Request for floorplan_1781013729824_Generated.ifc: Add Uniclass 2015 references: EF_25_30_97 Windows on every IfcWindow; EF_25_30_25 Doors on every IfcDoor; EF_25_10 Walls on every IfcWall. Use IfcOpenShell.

First a look at what the model holds.

```python
import ifcopenshell

model = ifcopenshell.open("floorplan_1781013729824_Generated.ifc")
print(model.schema)
print("classifications:", [c.Name for c in model.by_type("IfcClassification")])
for ifc_class in ("IfcDoor", "IfcRoof", "IfcStair", "IfcWall", "IfcWindow"):
    print(ifc_class, len(model.by_type(ifc_class)))
```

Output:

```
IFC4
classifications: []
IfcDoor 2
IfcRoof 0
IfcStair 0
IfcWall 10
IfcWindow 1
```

```python
import ifcopenshell
import ifcopenshell.api.classification

model = ifcopenshell.open("floorplan_1781013729824_Generated.ifc")

system = ifcopenshell.api.classification.add_classification(model, classification="Uniclass 2015")

codes = {
    "IfcWindow": ("EF_25_30_97", "Windows"),
    "IfcDoor": ("EF_25_30_25", "Doors"),
    "IfcWall": ("EF_25_10", "Walls"),
}
for ifc_class, (code, name) in codes.items():
    products = model.by_type(ifc_class)
    ifcopenshell.api.classification.add_reference(
        model, products=products, classification=system, identification=code, name=name
    )
    print(code, len(products))

model.write("floorplan_1781013729824_Generated_rev.ifc")
```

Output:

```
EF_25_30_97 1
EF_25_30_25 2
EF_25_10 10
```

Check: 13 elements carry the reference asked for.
